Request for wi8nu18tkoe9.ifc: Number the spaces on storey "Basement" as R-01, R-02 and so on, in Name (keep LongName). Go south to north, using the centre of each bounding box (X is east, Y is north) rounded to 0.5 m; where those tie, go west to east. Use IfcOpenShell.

First a look at what the model holds.

```python
import ifcopenshell
import ifcopenshell.util.element
import ifcopenshell.util.placement

model = ifcopenshell.open("wi8nu18tkoe9.ifc")
print(model.schema)
storey = next(s for s in model.by_type("IfcBuildingStorey") if s.Name == "Basement")
spaces = [e for e in ifcopenshell.util.element.get_decomposition(storey) if e.is_a("IfcSpace")]
for e in sorted(spaces, key=lambda e: e.id()):
    origin = ifcopenshell.util.placement.get_local_placement(e.ObjectPlacement)[:3, 3]
    print(e.id(), e.Name, e.LongName, origin.round(2) + 0.0, sep=" | ")
```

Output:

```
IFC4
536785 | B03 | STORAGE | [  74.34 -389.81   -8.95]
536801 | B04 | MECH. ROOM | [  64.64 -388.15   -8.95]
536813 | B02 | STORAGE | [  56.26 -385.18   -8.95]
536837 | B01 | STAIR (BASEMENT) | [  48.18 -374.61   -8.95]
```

```python
import ifcopenshell
import ifcopenshell.geom
import ifcopenshell.util.element
import ifcopenshell.util.shape

model = ifcopenshell.open("wi8nu18tkoe9.ifc")
settings = ifcopenshell.geom.settings()
settings.set("use-world-coords", True)


def centre(element):
    shape = ifcopenshell.geom.create_shape(settings, element)
    return ifcopenshell.util.shape.get_bbox_centroid(shape.geometry)


storey = next(s for s in model.by_type("IfcBuildingStorey") if s.Name == "Basement")
spaces = [e for e in ifcopenshell.util.element.get_decomposition(storey) if e.is_a("IfcSpace")]

# Insertion points can sit at a corner or the storey origin, so sort by the geometry (in metres).
centres = {e: centre(e) for e in spaces}
spaces.sort(key=lambda e: (round(centres[e][1] / 0.5), centres[e][0]))

for i, e in enumerate(spaces, start=1):
    number = f"R-{i:02d}"
    e.Name = number
    print(e.id(), number)

model.write("wi8nu18tkoe9_edited.ifc")
```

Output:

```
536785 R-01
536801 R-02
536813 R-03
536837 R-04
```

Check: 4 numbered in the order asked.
